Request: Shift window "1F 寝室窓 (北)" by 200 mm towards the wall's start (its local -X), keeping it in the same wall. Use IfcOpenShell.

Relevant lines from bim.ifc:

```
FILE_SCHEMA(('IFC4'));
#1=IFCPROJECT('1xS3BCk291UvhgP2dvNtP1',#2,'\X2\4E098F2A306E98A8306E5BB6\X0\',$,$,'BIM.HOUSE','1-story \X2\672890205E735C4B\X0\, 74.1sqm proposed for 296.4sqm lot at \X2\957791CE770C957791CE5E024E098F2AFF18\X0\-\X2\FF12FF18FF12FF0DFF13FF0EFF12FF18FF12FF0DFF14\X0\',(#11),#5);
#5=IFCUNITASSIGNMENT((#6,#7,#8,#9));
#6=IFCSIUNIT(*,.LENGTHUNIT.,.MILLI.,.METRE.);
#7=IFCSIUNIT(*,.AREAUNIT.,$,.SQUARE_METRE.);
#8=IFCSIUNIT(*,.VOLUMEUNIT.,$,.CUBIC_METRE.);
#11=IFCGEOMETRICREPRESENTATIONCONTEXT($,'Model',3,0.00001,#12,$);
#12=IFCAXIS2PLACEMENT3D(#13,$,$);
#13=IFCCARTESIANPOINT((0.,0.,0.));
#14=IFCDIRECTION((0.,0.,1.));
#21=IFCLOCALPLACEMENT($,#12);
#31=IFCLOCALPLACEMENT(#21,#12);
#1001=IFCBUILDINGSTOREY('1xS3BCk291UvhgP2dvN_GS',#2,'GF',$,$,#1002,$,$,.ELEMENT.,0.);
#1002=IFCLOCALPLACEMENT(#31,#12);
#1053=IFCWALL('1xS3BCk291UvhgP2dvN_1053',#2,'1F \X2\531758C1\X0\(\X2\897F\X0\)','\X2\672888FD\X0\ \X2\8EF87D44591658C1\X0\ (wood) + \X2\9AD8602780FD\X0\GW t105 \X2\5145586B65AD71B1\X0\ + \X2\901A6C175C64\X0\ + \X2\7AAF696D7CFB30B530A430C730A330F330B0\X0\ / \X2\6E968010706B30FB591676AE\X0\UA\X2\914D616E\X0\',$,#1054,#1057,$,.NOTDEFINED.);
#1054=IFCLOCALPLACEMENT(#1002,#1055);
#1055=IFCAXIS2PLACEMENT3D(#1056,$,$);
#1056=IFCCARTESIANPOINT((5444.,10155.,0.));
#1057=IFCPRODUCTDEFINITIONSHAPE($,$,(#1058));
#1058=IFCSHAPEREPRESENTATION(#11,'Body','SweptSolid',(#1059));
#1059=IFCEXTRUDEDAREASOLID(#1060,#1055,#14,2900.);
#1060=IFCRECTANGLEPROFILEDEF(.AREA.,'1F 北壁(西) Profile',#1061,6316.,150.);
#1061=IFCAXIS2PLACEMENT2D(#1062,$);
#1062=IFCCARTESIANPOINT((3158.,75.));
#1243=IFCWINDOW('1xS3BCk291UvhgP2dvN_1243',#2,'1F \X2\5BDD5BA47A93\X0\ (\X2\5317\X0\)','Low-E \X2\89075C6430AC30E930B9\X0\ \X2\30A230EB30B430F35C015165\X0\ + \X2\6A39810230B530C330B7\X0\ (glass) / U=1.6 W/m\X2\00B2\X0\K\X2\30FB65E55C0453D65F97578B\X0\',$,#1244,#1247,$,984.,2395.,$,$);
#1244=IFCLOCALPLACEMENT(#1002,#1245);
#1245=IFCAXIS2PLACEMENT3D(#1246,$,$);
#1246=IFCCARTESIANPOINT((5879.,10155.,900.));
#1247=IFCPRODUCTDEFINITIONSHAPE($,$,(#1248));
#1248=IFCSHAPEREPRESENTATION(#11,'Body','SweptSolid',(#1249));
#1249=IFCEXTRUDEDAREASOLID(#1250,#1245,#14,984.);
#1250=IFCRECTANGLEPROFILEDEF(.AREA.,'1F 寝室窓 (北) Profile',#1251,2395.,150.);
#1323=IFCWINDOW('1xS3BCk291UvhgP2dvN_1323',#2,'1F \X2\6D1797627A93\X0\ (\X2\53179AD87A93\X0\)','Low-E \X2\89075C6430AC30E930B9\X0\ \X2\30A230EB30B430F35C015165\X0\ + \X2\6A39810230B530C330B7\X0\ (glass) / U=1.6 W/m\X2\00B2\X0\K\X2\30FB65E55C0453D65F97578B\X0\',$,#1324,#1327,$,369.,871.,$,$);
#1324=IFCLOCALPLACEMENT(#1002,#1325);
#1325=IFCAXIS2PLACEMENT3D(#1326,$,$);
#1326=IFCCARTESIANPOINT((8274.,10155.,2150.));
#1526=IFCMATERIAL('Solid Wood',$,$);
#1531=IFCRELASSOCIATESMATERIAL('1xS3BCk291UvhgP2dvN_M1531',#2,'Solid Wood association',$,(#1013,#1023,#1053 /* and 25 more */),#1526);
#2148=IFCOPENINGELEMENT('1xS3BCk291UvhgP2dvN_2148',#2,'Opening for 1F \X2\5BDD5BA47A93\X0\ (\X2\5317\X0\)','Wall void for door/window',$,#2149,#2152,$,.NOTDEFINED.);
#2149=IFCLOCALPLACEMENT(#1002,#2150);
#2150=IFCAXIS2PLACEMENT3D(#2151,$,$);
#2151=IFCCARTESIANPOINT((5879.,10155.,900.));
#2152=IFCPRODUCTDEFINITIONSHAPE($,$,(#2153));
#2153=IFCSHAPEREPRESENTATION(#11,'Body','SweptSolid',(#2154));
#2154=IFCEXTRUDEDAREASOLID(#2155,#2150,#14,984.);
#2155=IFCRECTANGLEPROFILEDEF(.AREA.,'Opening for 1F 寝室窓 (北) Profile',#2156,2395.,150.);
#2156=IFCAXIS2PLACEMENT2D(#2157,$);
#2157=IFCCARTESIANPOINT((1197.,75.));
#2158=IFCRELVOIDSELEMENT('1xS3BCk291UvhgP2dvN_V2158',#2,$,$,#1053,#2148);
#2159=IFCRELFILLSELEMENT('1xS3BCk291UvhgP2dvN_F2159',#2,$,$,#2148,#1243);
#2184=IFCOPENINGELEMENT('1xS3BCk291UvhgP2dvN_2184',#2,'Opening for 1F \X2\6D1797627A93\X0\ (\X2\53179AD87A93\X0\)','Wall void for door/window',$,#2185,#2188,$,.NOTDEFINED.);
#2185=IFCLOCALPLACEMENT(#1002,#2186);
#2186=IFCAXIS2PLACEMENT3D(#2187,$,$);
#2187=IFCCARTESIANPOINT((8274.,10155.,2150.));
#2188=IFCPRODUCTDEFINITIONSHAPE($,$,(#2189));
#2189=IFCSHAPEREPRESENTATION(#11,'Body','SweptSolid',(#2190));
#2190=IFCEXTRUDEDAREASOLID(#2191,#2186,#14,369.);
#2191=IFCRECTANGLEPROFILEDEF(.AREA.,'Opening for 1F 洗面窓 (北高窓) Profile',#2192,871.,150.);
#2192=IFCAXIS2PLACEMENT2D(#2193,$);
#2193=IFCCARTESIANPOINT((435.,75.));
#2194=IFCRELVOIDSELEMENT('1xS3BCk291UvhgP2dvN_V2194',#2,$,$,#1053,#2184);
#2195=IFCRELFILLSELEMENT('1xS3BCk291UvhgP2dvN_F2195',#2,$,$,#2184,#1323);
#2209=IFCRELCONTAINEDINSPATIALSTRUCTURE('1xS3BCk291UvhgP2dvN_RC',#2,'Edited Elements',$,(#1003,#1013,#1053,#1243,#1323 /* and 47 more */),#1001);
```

```python
import ifcopenshell
import ifcopenshell.api.geometry
import ifcopenshell.util.placement
import ifcopenshell.util.unit

model = ifcopenshell.open("bim.ifc")
unit_scale = ifcopenshell.util.unit.calculate_unit_scale(model)

window = model.by_id(1243)
opening = window.FillsVoids[0].RelatingOpeningElement
wall = opening.VoidsElements[0].RelatingBuildingElement

wall_matrix = ifcopenshell.util.placement.get_local_placement(wall.ObjectPlacement)
shift = wall_matrix[:3, 0] * -0.2 / unit_scale
before = ifcopenshell.util.placement.get_local_placement(window.ObjectPlacement)[:3, 3].copy()

# The window is not placed relative to its opening, so move both.
for product in (opening, window):
    matrix = ifcopenshell.util.placement.get_local_placement(product.ObjectPlacement)
    matrix[:3, 3] += shift
    ifcopenshell.api.geometry.edit_object_placement(model, product=product, matrix=matrix, is_si=False)

after = ifcopenshell.util.placement.get_local_placement(window.ObjectPlacement)[:3, 3]
print("window moved by", (after - before).round(3) + 0.0)

model.write("bim_v2.ifc")
```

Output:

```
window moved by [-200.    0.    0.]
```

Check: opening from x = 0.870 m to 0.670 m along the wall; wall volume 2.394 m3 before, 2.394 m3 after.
